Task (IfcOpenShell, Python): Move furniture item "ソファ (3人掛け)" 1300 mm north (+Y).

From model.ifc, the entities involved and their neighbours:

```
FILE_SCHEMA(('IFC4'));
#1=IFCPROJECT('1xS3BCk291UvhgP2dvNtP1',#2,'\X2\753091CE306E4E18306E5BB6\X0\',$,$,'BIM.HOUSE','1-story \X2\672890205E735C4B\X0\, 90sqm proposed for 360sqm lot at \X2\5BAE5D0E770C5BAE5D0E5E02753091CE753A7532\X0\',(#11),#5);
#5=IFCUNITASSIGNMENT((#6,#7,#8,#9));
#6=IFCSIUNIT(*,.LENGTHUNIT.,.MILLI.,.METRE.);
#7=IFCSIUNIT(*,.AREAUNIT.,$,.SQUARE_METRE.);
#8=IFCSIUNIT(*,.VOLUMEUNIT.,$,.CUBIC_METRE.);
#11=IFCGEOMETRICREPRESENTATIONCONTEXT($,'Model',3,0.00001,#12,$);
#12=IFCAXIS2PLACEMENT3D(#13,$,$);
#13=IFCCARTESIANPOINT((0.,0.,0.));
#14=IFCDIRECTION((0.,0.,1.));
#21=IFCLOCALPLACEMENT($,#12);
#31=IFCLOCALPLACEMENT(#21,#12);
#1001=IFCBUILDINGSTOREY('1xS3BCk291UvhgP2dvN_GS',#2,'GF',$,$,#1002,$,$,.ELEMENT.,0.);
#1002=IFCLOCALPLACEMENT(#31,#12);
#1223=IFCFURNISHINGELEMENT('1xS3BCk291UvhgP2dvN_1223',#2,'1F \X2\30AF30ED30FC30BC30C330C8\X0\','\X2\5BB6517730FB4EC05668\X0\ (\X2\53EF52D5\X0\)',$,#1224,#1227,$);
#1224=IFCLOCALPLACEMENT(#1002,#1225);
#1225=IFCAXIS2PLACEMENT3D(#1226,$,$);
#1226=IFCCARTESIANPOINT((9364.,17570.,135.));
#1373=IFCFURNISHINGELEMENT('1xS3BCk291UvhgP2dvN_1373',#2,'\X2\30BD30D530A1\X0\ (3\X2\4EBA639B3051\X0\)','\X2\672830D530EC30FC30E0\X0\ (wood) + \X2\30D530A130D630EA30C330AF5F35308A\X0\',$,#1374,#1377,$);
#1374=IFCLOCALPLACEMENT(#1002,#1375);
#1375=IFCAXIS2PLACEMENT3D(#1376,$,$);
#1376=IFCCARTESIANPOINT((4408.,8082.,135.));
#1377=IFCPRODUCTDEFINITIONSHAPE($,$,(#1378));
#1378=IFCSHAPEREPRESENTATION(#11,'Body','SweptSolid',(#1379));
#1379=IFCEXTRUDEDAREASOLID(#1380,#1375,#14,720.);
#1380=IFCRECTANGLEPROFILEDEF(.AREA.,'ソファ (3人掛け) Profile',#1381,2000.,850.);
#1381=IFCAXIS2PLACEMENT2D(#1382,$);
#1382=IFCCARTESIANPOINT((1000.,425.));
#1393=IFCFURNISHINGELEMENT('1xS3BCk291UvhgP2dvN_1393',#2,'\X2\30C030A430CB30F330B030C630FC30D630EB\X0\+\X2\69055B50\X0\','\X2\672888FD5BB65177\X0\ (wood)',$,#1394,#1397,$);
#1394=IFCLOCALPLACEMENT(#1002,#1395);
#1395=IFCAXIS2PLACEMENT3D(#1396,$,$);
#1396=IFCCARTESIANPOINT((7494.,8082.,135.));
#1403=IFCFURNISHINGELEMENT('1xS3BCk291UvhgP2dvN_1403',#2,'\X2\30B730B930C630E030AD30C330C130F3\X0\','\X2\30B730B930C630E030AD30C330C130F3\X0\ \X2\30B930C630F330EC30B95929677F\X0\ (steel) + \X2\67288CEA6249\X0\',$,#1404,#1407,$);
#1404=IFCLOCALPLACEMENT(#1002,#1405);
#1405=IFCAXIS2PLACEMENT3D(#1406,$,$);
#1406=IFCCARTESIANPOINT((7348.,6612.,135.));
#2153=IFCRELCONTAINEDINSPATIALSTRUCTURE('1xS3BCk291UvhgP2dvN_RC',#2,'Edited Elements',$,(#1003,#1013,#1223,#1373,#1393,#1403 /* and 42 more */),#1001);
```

```python
import ifcopenshell
import ifcopenshell.api.geometry
import ifcopenshell.util.placement

model = ifcopenshell.open("model.ifc")

item = model.by_id(1373)
matrix = ifcopenshell.util.placement.get_local_placement(item.ObjectPlacement)
matrix[1, 3] += 1300.0
ifcopenshell.api.geometry.edit_object_placement(model, product=item, matrix=matrix, is_si=False)

print(ifcopenshell.util.placement.get_local_placement(item.ObjectPlacement).round(3) + 0.0)

model.write("model-out.ifc")
```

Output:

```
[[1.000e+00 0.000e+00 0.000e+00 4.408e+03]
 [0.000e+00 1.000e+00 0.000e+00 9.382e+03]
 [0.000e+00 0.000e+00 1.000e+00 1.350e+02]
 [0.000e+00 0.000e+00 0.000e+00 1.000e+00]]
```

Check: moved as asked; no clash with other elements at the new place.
